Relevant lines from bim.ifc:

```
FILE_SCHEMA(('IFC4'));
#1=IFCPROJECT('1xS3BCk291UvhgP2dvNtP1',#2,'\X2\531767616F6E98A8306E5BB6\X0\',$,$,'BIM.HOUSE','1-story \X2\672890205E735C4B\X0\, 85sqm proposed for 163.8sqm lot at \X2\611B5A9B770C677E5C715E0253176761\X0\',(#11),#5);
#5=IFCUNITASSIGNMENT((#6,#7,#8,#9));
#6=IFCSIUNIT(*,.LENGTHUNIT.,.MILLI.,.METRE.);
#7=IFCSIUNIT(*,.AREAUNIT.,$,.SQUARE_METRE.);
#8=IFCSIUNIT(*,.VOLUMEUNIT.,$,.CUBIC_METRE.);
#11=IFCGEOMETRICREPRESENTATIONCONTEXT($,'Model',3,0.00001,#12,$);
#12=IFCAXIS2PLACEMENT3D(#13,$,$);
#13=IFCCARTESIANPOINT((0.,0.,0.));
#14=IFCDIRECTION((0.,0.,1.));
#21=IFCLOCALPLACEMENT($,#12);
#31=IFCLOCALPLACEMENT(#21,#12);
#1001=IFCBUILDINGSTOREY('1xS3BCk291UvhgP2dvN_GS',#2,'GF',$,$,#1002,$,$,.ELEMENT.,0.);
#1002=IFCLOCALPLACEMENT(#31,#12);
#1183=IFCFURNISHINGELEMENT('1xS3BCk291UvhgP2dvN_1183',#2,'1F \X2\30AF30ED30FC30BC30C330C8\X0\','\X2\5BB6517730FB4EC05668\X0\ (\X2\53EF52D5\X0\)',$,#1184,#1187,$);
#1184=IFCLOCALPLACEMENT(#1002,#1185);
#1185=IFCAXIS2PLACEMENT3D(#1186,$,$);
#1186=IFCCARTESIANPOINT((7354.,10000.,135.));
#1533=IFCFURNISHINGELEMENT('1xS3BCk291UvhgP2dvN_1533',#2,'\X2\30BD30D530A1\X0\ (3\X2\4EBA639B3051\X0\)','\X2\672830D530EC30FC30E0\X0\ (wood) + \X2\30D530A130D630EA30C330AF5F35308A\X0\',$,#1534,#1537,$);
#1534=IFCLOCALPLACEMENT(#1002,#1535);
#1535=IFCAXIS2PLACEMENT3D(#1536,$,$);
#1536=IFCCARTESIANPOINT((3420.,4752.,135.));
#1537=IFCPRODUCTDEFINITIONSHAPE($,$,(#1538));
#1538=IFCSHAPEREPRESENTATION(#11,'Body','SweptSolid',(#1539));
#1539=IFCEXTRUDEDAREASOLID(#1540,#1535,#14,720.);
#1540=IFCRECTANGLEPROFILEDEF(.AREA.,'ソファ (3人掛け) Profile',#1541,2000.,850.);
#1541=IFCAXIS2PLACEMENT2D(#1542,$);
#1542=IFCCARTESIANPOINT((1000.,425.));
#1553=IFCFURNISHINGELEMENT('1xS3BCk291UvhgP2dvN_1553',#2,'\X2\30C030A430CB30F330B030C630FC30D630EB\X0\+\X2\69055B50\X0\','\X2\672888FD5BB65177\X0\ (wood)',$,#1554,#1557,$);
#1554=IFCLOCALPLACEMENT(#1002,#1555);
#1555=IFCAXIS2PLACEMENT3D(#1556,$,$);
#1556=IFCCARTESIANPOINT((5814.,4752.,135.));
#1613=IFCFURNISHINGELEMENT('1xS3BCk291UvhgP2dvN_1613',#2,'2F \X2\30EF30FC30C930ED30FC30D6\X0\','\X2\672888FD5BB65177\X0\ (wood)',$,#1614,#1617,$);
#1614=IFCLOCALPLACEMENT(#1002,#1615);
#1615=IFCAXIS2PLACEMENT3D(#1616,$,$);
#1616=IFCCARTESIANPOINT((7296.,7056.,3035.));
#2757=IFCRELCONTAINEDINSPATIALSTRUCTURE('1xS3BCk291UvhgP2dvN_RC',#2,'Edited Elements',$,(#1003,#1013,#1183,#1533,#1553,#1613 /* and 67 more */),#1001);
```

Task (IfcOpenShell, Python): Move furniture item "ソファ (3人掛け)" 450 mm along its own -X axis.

```python
import ifcopenshell
import ifcopenshell.api.geometry
import ifcopenshell.util.placement
import ifcopenshell.util.unit

model = ifcopenshell.open("bim.ifc")
unit_scale = ifcopenshell.util.unit.calculate_unit_scale(model)

item = model.by_guid("1xS3BCk291UvhgP2dvN_1533")
matrix = ifcopenshell.util.placement.get_local_placement(item.ObjectPlacement)
matrix[:3, 3] -= matrix[:3, 0] * 0.45 / unit_scale
ifcopenshell.api.geometry.edit_object_placement(model, product=item, matrix=matrix, is_si=False)

print(ifcopenshell.util.placement.get_local_placement(item.ObjectPlacement).round(3) + 0.0)

model.write("bim_v2.ifc")
```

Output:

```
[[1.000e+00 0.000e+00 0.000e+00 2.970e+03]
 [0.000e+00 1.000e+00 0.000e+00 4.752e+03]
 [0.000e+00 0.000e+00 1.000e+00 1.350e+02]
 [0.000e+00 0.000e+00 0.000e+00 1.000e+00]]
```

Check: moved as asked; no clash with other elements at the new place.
